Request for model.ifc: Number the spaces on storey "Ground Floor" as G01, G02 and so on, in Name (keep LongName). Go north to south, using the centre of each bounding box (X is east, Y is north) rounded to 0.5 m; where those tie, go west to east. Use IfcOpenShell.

First a look at what the model holds.

```python
import ifcopenshell
import ifcopenshell.util.element
import ifcopenshell.util.placement

model = ifcopenshell.open("model.ifc")
print(model.schema)
storey = next(s for s in model.by_type("IfcBuildingStorey") if s.Name == "Ground Floor")
spaces = [e for e in ifcopenshell.util.element.get_decomposition(storey) if e.is_a("IfcSpace")]
for e in sorted(spaces, key=lambda e: e.id()):
    origin = ifcopenshell.util.placement.get_local_placement(e.ObjectPlacement)[:3, 3]
    print(e.id(), e.Name, e.LongName, origin.round(2) + 0.0, sep=" | ")
```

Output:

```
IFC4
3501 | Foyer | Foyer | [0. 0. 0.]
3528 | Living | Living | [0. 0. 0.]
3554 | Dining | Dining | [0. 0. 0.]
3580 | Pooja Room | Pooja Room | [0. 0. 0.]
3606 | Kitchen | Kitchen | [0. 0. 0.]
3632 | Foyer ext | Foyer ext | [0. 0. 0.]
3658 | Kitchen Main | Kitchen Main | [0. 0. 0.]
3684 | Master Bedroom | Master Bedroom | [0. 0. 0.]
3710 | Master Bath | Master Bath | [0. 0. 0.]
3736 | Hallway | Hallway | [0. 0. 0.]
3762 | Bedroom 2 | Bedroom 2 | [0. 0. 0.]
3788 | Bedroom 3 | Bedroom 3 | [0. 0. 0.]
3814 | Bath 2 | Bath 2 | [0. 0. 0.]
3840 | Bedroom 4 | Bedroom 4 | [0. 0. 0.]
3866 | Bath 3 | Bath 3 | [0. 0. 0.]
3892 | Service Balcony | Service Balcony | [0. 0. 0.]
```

```python
import ifcopenshell
import ifcopenshell.geom
import ifcopenshell.util.element
import ifcopenshell.util.shape

model = ifcopenshell.open("model.ifc")
settings = ifcopenshell.geom.settings()
settings.set("use-world-coords", True)


def centre(element):
    shape = ifcopenshell.geom.create_shape(settings, element)
    return ifcopenshell.util.shape.get_bbox_centroid(shape.geometry)


storey = next(s for s in model.by_type("IfcBuildingStorey") if s.Name == "Ground Floor")
spaces = [e for e in ifcopenshell.util.element.get_decomposition(storey) if e.is_a("IfcSpace")]

# Insertion points can sit at a corner or the storey origin, so sort by the geometry (in metres).
centres = {e: centre(e) for e in spaces}
spaces.sort(key=lambda e: (-round(centres[e][1] / 0.5), centres[e][0]))

for i, e in enumerate(spaces, start=1):
    number = f"G{i:02d}"
    e.Name = number
    print(e.id(), number)

model.write("model_updated.ifc")
```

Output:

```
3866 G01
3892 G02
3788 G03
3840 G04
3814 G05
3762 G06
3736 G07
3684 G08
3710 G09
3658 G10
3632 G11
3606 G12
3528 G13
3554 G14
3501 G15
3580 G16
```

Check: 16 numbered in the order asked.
